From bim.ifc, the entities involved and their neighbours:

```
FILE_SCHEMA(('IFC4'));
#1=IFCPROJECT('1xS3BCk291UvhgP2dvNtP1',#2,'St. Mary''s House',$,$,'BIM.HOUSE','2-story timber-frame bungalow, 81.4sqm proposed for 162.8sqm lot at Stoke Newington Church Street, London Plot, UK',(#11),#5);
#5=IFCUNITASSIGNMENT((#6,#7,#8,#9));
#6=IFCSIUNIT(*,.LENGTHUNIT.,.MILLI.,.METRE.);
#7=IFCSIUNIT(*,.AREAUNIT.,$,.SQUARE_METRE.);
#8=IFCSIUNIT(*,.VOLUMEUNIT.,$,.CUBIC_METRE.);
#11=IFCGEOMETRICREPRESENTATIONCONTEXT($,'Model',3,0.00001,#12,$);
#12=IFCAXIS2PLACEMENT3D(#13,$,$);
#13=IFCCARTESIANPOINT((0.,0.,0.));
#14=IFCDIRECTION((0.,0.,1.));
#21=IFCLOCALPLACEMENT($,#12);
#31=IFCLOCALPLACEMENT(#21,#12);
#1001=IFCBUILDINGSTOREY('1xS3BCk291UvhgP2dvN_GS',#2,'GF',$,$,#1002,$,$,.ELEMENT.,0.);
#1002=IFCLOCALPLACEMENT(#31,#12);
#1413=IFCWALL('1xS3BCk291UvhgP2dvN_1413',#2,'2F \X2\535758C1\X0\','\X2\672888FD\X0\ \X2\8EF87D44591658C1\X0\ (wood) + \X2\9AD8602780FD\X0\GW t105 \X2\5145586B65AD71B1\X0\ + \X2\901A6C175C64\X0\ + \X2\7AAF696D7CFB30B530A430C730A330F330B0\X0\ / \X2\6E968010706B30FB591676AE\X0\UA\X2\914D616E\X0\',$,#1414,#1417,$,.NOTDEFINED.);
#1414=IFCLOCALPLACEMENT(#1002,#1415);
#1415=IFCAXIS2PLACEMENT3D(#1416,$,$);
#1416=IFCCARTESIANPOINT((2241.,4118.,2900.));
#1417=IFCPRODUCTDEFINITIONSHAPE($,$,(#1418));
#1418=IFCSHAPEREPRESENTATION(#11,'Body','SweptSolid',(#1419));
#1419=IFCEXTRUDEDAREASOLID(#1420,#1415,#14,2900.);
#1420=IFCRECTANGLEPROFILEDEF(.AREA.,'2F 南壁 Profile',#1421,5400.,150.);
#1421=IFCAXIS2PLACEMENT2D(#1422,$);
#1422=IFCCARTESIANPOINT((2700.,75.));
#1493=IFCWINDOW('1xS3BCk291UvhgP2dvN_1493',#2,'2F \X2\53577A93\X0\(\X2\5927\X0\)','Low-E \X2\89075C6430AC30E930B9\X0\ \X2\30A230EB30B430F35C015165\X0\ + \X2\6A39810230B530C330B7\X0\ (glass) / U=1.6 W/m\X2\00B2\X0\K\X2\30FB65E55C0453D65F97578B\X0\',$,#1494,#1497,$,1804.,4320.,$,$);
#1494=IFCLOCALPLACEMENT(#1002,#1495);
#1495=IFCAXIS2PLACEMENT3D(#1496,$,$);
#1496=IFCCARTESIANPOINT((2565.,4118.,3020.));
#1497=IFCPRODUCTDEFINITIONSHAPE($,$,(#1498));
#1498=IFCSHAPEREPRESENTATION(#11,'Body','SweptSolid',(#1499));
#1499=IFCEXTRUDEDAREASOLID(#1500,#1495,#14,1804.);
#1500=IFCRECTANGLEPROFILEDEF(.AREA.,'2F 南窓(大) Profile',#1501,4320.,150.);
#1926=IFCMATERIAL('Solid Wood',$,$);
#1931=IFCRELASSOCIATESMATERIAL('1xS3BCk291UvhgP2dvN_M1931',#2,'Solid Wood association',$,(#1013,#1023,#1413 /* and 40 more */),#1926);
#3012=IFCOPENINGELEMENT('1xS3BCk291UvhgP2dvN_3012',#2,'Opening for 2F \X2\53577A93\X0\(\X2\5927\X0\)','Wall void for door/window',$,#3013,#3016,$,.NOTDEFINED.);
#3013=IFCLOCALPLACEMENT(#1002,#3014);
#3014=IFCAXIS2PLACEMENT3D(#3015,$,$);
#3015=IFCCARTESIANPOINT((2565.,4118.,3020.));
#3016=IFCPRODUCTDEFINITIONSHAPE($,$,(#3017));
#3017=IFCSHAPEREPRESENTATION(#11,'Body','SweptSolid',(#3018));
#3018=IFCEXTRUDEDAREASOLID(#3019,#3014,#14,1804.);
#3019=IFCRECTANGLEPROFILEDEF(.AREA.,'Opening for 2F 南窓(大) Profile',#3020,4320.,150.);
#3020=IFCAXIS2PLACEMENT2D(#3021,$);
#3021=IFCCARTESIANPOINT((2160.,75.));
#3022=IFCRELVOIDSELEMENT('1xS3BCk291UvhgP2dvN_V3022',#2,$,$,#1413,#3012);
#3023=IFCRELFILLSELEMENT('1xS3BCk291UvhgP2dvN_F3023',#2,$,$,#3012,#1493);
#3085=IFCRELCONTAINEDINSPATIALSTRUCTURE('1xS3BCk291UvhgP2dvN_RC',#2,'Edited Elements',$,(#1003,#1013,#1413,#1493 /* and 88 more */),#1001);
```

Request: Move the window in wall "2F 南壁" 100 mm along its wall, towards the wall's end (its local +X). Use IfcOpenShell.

```python
import ifcopenshell
import ifcopenshell.api.geometry
import ifcopenshell.util.placement

model = ifcopenshell.open("bim.ifc")

window = model.by_guid("1xS3BCk291UvhgP2dvN_1493")
opening = window.FillsVoids[0].RelatingOpeningElement
wall = opening.VoidsElements[0].RelatingBuildingElement

wall_matrix = ifcopenshell.util.placement.get_local_placement(wall.ObjectPlacement)
shift = wall_matrix[:3, 0] * 100.0
before = ifcopenshell.util.placement.get_local_placement(window.ObjectPlacement)[:3, 3].copy()

# The window is not placed relative to its opening, so move both.
for product in (opening, window):
    matrix = ifcopenshell.util.placement.get_local_placement(product.ObjectPlacement)
    matrix[:3, 3] += shift
    ifcopenshell.api.geometry.edit_object_placement(model, product=product, matrix=matrix, is_si=False)

after = ifcopenshell.util.placement.get_local_placement(window.ObjectPlacement)[:3, 3]
print("window moved by", (after - before).round(3) + 0.0)

model.write("bim_updated.ifc")
```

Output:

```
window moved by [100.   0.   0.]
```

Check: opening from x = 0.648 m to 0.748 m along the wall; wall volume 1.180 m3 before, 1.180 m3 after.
